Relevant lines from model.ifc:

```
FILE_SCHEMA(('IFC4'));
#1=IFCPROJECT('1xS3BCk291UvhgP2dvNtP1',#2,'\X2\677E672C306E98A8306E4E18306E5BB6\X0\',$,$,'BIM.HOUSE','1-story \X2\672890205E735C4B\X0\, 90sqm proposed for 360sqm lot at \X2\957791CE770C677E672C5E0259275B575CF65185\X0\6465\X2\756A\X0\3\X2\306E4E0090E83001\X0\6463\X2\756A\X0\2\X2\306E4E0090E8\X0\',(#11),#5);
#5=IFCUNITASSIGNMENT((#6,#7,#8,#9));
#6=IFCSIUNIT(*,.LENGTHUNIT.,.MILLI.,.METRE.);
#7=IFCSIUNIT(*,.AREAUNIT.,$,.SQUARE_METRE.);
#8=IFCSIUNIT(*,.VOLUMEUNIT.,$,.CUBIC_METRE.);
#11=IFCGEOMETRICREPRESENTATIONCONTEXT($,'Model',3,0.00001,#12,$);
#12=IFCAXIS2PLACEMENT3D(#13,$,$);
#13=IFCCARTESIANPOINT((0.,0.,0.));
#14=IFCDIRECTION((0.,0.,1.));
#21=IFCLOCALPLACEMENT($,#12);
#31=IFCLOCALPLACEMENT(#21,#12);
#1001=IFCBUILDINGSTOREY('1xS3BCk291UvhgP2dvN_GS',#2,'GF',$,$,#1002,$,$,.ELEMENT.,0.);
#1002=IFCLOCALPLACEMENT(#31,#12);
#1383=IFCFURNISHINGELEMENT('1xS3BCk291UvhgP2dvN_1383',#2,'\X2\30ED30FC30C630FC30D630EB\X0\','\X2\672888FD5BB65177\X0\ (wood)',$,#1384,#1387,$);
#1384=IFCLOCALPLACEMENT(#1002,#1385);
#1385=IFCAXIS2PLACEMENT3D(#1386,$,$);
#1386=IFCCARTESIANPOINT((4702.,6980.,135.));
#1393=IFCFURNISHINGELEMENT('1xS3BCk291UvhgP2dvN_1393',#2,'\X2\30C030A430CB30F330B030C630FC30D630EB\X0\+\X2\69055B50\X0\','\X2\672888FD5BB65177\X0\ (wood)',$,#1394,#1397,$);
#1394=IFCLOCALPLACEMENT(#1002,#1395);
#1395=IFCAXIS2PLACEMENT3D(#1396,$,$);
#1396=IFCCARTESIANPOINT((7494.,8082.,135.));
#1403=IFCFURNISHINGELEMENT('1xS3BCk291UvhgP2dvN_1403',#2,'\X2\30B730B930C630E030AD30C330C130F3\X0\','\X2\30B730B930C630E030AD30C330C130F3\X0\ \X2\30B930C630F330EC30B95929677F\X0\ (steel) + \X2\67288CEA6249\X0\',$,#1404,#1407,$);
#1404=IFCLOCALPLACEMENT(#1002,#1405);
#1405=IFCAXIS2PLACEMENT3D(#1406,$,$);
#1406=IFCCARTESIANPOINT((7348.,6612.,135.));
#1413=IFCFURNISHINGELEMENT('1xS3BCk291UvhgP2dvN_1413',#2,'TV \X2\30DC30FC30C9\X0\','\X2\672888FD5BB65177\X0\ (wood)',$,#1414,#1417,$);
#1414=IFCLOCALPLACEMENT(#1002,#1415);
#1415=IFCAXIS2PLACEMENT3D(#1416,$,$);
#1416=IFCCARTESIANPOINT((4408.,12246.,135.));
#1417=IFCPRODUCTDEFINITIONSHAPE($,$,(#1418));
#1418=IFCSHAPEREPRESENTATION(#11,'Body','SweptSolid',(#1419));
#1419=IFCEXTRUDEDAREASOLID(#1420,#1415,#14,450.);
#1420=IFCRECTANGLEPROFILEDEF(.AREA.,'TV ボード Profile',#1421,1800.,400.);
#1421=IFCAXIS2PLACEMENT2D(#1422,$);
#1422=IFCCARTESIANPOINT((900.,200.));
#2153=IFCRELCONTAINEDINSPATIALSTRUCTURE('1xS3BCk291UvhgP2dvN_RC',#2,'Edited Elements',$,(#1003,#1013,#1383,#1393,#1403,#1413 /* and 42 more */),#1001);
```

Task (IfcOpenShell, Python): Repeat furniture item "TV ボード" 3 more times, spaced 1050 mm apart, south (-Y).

```python
import numpy as np
import ifcopenshell
import ifcopenshell.api.geometry
import ifcopenshell.api.root
import ifcopenshell.util.element
import ifcopenshell.util.placement

model = ifcopenshell.open("model.ifc")


def reuse_history(source, copy):
    """copy_class also copies each property set's owner history, people and application; keep the originals."""
    for rel in copy.IsDefinedBy:
        if rel.is_a("IfcRelDefinesByProperties") and (history := rel.RelatingPropertyDefinition.OwnerHistory):
            rel.RelatingPropertyDefinition.OwnerHistory = source.OwnerHistory
            ifcopenshell.util.element.remove_deep2(model, history)


source = model.by_guid("1xS3BCk291UvhgP2dvN_1413")
base = ifcopenshell.util.placement.get_local_placement(source.ObjectPlacement)
step = np.array([0.0, -1.0, 0.0]) * 1050.0

for i in range(1, 4):
    copy = ifcopenshell.api.root.copy_class(model, product=source)
    copy.Representation = ifcopenshell.util.element.copy_deep(
        model, source.Representation, exclude=["IfcGeometricRepresentationContext", "IfcRepresentationMap"]
    )
    reuse_history(source, copy)
    matrix = base.copy()
    matrix[:3, 3] += i * step
    print("added at", matrix[:3, 3].round(3) + 0.0)
    ifcopenshell.api.geometry.edit_object_placement(model, product=copy, matrix=matrix, is_si=False)

model.write("model_v2.ifc")
```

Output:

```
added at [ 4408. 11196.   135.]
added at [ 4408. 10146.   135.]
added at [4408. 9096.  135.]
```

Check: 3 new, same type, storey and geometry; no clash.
